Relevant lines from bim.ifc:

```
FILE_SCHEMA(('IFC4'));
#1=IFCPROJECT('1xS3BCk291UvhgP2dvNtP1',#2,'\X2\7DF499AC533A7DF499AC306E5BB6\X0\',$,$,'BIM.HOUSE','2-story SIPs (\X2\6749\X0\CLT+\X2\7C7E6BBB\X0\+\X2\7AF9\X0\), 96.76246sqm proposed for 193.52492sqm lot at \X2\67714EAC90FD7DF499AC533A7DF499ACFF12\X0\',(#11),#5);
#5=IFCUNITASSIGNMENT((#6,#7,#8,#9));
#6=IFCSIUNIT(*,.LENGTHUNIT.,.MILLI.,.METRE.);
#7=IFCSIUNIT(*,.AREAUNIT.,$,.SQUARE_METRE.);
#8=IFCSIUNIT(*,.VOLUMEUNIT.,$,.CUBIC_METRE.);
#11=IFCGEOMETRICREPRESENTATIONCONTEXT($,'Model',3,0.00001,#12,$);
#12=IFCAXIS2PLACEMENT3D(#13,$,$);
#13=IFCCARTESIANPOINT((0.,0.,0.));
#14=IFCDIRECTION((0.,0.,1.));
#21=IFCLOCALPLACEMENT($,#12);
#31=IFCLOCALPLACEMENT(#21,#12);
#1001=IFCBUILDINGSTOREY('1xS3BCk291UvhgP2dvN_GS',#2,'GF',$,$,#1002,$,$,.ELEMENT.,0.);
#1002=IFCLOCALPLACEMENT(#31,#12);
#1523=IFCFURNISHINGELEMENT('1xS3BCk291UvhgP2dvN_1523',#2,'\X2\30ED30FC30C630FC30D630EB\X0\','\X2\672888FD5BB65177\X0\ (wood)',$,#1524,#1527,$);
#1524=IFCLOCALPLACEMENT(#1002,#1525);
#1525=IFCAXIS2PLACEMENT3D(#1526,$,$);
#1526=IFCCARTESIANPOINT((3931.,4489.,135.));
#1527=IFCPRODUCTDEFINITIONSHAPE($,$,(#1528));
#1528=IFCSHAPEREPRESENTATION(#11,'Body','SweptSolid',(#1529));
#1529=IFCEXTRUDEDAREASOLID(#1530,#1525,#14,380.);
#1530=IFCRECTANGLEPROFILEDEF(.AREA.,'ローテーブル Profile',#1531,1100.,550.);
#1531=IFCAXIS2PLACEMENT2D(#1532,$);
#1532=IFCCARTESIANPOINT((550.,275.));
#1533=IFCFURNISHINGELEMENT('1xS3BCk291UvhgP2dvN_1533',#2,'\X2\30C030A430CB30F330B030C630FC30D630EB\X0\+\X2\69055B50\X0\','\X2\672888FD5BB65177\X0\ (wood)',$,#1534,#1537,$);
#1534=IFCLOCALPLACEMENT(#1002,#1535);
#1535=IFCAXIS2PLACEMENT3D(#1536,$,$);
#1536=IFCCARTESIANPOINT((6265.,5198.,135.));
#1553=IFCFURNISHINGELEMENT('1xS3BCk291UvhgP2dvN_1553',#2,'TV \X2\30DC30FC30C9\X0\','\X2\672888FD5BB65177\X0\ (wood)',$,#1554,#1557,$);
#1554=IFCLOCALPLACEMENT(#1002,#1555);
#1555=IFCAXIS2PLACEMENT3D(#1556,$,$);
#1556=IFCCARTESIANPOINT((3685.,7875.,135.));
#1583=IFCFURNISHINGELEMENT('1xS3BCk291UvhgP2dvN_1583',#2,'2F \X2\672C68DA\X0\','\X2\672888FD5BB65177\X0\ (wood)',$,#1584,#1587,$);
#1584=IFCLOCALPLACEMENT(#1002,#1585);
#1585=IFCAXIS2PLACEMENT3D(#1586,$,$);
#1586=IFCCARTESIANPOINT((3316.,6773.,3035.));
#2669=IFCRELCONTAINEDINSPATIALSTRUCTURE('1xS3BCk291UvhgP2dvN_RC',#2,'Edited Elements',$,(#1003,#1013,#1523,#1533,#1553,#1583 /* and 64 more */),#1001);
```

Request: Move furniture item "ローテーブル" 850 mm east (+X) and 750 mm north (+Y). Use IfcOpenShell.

```python
import ifcopenshell
import ifcopenshell.api.geometry
import ifcopenshell.util.placement
import ifcopenshell.util.unit

model = ifcopenshell.open("bim.ifc")
unit_scale = ifcopenshell.util.unit.calculate_unit_scale(model)

item = model.by_guid("1xS3BCk291UvhgP2dvN_1523")
matrix = ifcopenshell.util.placement.get_local_placement(item.ObjectPlacement)
matrix[0, 3] += 0.85 / unit_scale
matrix[1, 3] += 0.75 / unit_scale
ifcopenshell.api.geometry.edit_object_placement(model, product=item, matrix=matrix, is_si=False)

print(ifcopenshell.util.placement.get_local_placement(item.ObjectPlacement).round(3) + 0.0)

model.write("bim_v2.ifc")
```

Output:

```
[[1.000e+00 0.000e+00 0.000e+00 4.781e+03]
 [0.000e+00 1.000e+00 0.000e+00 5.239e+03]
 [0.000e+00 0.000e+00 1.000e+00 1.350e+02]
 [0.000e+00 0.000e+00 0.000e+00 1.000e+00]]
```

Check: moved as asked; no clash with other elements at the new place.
